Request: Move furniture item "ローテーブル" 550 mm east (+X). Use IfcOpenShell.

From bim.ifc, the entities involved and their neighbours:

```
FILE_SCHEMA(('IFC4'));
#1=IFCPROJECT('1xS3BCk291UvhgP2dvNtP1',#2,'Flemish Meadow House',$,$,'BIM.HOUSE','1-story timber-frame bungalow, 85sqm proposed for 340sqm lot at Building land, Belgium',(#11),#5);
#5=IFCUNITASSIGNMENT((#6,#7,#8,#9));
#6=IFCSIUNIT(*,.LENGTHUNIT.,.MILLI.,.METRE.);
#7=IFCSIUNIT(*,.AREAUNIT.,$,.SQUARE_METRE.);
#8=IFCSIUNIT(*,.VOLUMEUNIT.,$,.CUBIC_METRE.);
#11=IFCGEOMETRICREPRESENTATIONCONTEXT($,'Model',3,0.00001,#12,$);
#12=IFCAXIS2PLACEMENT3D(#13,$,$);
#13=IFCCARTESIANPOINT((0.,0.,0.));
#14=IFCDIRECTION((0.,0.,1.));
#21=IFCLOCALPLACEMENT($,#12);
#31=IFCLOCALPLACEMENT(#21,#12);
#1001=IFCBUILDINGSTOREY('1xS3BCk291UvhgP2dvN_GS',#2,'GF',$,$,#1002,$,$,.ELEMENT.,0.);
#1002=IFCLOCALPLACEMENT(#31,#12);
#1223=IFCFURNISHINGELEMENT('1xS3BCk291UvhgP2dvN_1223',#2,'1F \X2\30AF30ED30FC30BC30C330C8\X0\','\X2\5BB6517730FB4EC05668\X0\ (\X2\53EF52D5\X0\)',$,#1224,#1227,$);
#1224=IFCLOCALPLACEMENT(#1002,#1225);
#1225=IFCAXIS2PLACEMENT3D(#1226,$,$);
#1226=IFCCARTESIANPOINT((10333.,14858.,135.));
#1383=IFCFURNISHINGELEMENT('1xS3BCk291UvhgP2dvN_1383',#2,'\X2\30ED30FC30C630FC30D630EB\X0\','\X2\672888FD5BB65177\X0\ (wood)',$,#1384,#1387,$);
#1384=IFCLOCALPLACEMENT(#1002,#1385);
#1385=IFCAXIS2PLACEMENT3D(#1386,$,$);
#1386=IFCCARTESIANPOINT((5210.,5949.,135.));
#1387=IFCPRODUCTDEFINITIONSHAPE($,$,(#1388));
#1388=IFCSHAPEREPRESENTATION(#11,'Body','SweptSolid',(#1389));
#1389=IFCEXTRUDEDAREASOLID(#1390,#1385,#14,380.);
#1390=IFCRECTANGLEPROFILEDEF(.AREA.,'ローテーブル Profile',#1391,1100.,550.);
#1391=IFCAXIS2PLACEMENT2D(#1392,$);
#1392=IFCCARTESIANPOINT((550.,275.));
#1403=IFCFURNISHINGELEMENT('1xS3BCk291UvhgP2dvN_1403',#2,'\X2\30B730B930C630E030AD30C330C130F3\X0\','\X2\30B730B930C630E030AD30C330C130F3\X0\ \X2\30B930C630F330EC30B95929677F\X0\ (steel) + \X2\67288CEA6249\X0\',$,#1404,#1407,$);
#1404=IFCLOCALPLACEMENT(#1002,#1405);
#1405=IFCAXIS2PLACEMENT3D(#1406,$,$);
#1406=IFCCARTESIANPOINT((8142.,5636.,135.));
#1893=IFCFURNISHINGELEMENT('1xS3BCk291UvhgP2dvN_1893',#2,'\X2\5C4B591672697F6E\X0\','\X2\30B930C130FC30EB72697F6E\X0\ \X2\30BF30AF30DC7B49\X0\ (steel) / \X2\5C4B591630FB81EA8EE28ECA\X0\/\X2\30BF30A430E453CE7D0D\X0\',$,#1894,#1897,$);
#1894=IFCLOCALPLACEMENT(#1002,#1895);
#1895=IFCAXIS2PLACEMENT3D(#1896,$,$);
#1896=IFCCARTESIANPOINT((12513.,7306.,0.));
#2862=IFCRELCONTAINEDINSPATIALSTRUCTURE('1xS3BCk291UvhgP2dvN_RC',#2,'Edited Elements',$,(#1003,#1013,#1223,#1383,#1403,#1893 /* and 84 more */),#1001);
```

```python
import ifcopenshell
import ifcopenshell.api.geometry
import ifcopenshell.util.placement

model = ifcopenshell.open("bim.ifc")

item = model.by_id(1383)
matrix = ifcopenshell.util.placement.get_local_placement(item.ObjectPlacement)
matrix[0, 3] += 550.0
ifcopenshell.api.geometry.edit_object_placement(model, product=item, matrix=matrix, is_si=False)

print(ifcopenshell.util.placement.get_local_placement(item.ObjectPlacement).round(3) + 0.0)

model.write("bim_v2.ifc")
```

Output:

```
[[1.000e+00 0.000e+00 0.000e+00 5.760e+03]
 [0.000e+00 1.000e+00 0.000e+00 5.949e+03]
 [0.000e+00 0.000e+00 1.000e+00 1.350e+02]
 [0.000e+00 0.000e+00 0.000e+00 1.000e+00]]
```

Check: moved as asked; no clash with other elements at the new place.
